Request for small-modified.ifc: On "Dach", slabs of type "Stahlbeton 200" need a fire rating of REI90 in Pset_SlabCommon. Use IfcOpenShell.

First a look at what the model holds.

```python
import ifcopenshell
import ifcopenshell.util.element

model = ifcopenshell.open("small-modified.ifc")
print(model.schema)
storey = next(s for s in model.by_type("IfcBuildingStorey") if s.Name == "Dach")
slabs = [e for e in ifcopenshell.util.element.get_decomposition(storey) if e.is_a("IfcSlab")]
seen = {}
for e in slabs:
    element_type = ifcopenshell.util.element.get_type(e)
    key = (element_type.Name if element_type != e and element_type else None, ifcopenshell.util.element.get_pset(e, "Pset_SlabCommon", "FireRating"))
    seen[key] = seen.get(key, 0) + 1
for (name, value), count in sorted(seen.items(), key=str):
    print(count, "x", name, "|", value)
```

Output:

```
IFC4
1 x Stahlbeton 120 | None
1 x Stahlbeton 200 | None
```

```python
import ifcopenshell
import ifcopenshell.api.pset
import ifcopenshell.util.element

model = ifcopenshell.open("small-modified.ifc")

storey = next(s for s in model.by_type("IfcBuildingStorey") if s.Name == "Dach")
slabs = [e for e in ifcopenshell.util.element.get_decomposition(storey) if e.is_a("IfcSlab")]

count = 0
for e in slabs:
    element_type = ifcopenshell.util.element.get_type(e)
    if element_type in (None, e) or element_type.Name != "Stahlbeton 200":
        continue
    # add_pset returns the element's existing set when there is one.
    pset = ifcopenshell.api.pset.add_pset(model, product=e, name="Pset_SlabCommon")
    ifcopenshell.api.pset.edit_pset(model, pset=pset, properties={"FireRating": "REI90"})
    count += 1

print(count, "slabs updated")

model.write("small-modified_rev.ifc")
```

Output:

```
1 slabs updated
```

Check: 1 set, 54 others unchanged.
